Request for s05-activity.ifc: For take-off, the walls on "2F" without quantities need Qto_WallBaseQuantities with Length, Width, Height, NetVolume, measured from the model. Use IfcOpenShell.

First a look at what the model holds.

```python
import ifcopenshell
import ifcopenshell.util.element
import ifcopenshell.util.unit

model = ifcopenshell.open("s05-activity.ifc")
print(model.schema)
for unit_type in ("LENGTHUNIT", "AREAUNIT", "VOLUMEUNIT"):
    print(unit_type, ifcopenshell.util.unit.calculate_unit_scale(model, unit_type))
storey = next(s for s in model.by_type("IfcBuildingStorey") if s.Name == "2F")
walls = [e for e in ifcopenshell.util.element.get_decomposition(storey) if e.is_a("IfcWall")]
for e in sorted(walls, key=lambda e: e.id()):
    print(e.id(), e.is_a(), e.Name, list(ifcopenshell.util.element.get_psets(e, qtos_only=True)), sep=" | ")
```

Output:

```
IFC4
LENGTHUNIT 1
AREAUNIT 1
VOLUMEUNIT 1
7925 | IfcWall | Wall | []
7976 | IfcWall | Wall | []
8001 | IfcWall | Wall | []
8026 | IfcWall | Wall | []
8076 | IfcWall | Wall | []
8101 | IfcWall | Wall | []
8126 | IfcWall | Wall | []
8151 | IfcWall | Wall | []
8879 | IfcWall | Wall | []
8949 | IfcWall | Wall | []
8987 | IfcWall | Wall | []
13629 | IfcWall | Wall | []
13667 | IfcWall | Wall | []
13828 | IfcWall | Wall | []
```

```python
import ifcopenshell
import ifcopenshell.api.pset
import ifcopenshell.geom
import ifcopenshell.util.element
import ifcopenshell.util.shape
import ifcopenshell.util.unit

model = ifcopenshell.open("s05-activity.ifc")
unit_scale = ifcopenshell.util.unit.calculate_unit_scale(model)
volume_scale = ifcopenshell.util.unit.calculate_unit_scale(model, "VOLUMEUNIT")
settings = ifcopenshell.geom.settings()

storey = next(s for s in model.by_type("IfcBuildingStorey") if s.Name == "2F")
walls = [e for e in ifcopenshell.util.element.get_decomposition(storey) if e.is_a("IfcWall")]

for e in sorted(walls, key=lambda e: e.id()):
    if ifcopenshell.util.element.get_psets(e, qtos_only=True, should_inherit=False):
        continue
    # Geometry comes back in metres, in the element's own axes.
    shape = ifcopenshell.geom.create_shape(settings, e)
    values = {
        "Length": ifcopenshell.util.shape.get_x(shape.geometry) / unit_scale,
        "Width": ifcopenshell.util.shape.get_y(shape.geometry) / unit_scale,
        "Height": ifcopenshell.util.shape.get_z(shape.geometry) / unit_scale,
        "NetVolume": ifcopenshell.util.shape.get_volume(shape.geometry) / volume_scale,
    }
    qto = ifcopenshell.api.pset.add_qto(model, product=e, name="Qto_WallBaseQuantities")
    ifcopenshell.api.pset.edit_qto(model, qto=qto, properties=values)
    print(e.id(), {k: round(v, 3) for k, v in values.items()})

model.write("s05-activity_updated.ifc")
```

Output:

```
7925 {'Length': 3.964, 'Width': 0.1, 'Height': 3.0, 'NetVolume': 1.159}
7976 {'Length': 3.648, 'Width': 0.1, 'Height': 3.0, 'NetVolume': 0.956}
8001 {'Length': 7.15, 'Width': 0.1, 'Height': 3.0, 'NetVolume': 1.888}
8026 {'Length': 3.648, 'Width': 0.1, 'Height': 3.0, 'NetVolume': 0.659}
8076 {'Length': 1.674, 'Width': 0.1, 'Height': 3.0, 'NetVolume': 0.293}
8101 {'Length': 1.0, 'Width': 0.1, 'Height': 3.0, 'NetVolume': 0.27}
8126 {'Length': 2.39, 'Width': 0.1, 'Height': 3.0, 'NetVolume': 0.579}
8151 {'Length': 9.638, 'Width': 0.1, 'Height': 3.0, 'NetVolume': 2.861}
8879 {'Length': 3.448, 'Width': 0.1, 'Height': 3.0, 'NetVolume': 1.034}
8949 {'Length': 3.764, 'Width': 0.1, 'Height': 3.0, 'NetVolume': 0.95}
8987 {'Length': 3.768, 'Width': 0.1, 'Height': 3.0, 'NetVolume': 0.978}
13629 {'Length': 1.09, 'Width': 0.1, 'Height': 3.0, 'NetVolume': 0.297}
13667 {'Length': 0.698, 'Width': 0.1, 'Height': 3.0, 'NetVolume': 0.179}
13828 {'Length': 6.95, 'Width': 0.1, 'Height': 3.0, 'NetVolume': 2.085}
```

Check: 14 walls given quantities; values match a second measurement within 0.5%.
